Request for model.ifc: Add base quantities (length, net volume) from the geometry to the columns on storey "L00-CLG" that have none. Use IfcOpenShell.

First a look at what the model holds.

```python
import ifcopenshell
import ifcopenshell.util.element
import ifcopenshell.util.unit

model = ifcopenshell.open("model.ifc")
print(model.schema)
for unit_type in ("LENGTHUNIT", "AREAUNIT", "VOLUMEUNIT"):
    print(unit_type, ifcopenshell.util.unit.calculate_unit_scale(model, unit_type))
storey = next(s for s in model.by_type("IfcBuildingStorey") if s.Name == "L00-CLG")
columns = [e for e in ifcopenshell.util.element.get_decomposition(storey) if e.is_a("IfcColumn")]
for e in sorted(columns, key=lambda e: e.id()):
    print(e.id(), e.is_a(), e.Name, list(ifcopenshell.util.element.get_psets(e, qtos_only=True)), sep=" | ")
```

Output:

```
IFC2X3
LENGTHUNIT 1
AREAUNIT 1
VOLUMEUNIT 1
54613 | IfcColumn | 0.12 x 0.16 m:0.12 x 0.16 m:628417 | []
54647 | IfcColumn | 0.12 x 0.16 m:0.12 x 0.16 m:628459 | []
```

```python
import ifcopenshell
import ifcopenshell.api.pset
import ifcopenshell.geom
import ifcopenshell.util.element
import ifcopenshell.util.shape
import ifcopenshell.util.unit

model = ifcopenshell.open("model.ifc")
unit_scale = ifcopenshell.util.unit.calculate_unit_scale(model)
volume_scale = ifcopenshell.util.unit.calculate_unit_scale(model, "VOLUMEUNIT")
settings = ifcopenshell.geom.settings()

storey = next(s for s in model.by_type("IfcBuildingStorey") if s.Name == "L00-CLG")
columns = [e for e in ifcopenshell.util.element.get_decomposition(storey) if e.is_a("IfcColumn")]

for e in sorted(columns, key=lambda e: e.id()):
    if ifcopenshell.util.element.get_psets(e, qtos_only=True, should_inherit=False):
        continue
    # Geometry comes back in metres, in the element's own axes.
    shape = ifcopenshell.geom.create_shape(settings, e)
    values = {
        "Length": ifcopenshell.util.shape.get_z(shape.geometry) / unit_scale,
        "NetVolume": ifcopenshell.util.shape.get_volume(shape.geometry) / volume_scale,
    }
    qto = ifcopenshell.api.pset.add_qto(model, product=e, name="BaseQuantities")
    ifcopenshell.api.pset.edit_qto(model, qto=qto, properties=values)
    print(e.id(), {k: round(v, 3) for k, v in values.items()})

model.write("model_v2.ifc")
```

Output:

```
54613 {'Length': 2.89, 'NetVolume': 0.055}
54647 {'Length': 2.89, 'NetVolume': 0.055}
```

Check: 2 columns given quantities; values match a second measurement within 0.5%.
